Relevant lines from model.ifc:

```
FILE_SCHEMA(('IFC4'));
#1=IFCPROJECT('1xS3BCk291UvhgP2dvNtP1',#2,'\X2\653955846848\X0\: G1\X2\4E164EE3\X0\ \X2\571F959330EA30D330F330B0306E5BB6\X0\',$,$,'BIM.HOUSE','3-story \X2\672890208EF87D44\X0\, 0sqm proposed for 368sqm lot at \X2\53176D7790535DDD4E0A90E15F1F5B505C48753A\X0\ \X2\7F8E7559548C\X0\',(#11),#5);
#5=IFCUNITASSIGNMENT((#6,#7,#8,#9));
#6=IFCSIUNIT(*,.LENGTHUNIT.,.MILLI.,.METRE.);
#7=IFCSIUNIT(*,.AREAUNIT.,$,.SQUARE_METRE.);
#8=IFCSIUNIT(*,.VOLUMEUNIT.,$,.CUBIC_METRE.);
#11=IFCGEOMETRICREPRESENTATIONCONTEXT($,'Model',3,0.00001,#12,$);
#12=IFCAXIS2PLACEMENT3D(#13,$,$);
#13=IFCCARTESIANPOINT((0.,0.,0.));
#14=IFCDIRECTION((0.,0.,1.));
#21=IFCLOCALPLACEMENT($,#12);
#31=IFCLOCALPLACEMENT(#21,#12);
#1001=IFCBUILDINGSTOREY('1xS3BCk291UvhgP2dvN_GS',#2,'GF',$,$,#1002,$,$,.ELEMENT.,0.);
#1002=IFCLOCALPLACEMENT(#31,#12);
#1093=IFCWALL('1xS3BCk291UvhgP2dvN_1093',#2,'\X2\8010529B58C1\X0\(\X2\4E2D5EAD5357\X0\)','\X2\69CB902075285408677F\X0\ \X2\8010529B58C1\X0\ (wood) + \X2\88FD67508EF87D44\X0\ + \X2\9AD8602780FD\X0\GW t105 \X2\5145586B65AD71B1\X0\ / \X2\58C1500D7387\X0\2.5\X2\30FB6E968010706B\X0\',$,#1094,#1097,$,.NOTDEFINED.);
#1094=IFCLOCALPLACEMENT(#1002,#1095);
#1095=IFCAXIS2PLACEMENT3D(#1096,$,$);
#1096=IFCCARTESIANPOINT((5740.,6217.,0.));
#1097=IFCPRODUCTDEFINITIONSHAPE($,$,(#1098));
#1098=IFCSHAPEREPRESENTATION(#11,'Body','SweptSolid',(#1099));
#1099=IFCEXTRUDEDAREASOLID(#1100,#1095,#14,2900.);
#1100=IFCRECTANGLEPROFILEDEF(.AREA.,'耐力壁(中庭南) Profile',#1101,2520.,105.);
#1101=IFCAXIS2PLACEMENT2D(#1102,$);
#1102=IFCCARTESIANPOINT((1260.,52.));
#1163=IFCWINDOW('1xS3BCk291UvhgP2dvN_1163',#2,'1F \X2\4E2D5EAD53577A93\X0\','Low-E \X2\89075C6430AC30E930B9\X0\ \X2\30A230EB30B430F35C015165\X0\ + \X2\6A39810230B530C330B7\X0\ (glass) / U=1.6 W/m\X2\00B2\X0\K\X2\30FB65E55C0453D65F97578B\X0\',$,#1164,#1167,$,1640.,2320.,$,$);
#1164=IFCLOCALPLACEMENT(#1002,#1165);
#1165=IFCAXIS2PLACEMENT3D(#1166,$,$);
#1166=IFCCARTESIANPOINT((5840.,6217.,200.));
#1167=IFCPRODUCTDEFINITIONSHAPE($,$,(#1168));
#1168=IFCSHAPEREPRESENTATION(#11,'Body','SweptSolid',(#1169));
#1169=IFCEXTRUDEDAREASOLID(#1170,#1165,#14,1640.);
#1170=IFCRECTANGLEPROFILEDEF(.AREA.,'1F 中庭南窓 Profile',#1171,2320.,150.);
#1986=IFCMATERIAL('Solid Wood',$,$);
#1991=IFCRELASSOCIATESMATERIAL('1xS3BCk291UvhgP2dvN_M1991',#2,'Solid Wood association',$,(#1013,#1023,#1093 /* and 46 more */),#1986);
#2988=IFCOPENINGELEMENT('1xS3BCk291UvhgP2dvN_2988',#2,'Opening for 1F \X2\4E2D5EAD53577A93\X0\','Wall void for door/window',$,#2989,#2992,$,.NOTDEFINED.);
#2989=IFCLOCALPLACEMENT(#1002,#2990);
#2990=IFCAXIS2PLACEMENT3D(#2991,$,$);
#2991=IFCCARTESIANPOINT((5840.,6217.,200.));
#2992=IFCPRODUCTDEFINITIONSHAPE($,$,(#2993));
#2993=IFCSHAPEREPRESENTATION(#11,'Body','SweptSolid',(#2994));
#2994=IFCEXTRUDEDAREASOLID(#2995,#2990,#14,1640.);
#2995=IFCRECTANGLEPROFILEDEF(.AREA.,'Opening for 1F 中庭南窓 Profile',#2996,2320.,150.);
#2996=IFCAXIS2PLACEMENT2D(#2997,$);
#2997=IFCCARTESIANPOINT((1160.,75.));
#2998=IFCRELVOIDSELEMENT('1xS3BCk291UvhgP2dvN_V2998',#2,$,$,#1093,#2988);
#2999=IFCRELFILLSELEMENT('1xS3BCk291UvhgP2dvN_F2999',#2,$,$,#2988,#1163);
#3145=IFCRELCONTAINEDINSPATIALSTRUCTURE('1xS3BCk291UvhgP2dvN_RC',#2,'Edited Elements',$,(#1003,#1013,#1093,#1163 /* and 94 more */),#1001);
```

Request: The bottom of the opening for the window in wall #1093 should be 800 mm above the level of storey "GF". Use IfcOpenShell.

```python
import numpy as np
import ifcopenshell
import ifcopenshell.api.geometry
import ifcopenshell.geom
import ifcopenshell.util.element
import ifcopenshell.util.placement
import ifcopenshell.util.shape
import ifcopenshell.util.unit

model = ifcopenshell.open("model.ifc")
unit_scale = ifcopenshell.util.unit.calculate_unit_scale(model)

window = model.by_guid("1xS3BCk291UvhgP2dvN_1163")
opening = window.FillsVoids[0].RelatingOpeningElement
storey = ifcopenshell.util.element.get_container(window, ifc_class="IfcBuildingStorey")
level = ifcopenshell.util.placement.get_local_placement(storey.ObjectPlacement)[2, 3]

# The opening's origin need not be at the sill, so measure its lowest point.
shape = ifcopenshell.geom.create_shape(ifcopenshell.geom.settings(), opening)
bottom = ifcopenshell.util.shape.get_shape_bottom_elevation(shape, shape.geometry) / unit_scale
dz = level + 0.8 / unit_scale - bottom

shift = np.array([0.0, 0.0, dz])
# The window is not placed relative to its opening, so move both.
for product in (opening, window):
    matrix = ifcopenshell.util.placement.get_local_placement(product.ObjectPlacement)
    matrix[:3, 3] += shift
    ifcopenshell.api.geometry.edit_object_placement(model, product=product, matrix=matrix, is_si=False)

print(f"moved by {dz * unit_scale:+.3f} m")

model.write("model_rev.ifc")
```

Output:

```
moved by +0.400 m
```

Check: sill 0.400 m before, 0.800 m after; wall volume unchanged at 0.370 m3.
